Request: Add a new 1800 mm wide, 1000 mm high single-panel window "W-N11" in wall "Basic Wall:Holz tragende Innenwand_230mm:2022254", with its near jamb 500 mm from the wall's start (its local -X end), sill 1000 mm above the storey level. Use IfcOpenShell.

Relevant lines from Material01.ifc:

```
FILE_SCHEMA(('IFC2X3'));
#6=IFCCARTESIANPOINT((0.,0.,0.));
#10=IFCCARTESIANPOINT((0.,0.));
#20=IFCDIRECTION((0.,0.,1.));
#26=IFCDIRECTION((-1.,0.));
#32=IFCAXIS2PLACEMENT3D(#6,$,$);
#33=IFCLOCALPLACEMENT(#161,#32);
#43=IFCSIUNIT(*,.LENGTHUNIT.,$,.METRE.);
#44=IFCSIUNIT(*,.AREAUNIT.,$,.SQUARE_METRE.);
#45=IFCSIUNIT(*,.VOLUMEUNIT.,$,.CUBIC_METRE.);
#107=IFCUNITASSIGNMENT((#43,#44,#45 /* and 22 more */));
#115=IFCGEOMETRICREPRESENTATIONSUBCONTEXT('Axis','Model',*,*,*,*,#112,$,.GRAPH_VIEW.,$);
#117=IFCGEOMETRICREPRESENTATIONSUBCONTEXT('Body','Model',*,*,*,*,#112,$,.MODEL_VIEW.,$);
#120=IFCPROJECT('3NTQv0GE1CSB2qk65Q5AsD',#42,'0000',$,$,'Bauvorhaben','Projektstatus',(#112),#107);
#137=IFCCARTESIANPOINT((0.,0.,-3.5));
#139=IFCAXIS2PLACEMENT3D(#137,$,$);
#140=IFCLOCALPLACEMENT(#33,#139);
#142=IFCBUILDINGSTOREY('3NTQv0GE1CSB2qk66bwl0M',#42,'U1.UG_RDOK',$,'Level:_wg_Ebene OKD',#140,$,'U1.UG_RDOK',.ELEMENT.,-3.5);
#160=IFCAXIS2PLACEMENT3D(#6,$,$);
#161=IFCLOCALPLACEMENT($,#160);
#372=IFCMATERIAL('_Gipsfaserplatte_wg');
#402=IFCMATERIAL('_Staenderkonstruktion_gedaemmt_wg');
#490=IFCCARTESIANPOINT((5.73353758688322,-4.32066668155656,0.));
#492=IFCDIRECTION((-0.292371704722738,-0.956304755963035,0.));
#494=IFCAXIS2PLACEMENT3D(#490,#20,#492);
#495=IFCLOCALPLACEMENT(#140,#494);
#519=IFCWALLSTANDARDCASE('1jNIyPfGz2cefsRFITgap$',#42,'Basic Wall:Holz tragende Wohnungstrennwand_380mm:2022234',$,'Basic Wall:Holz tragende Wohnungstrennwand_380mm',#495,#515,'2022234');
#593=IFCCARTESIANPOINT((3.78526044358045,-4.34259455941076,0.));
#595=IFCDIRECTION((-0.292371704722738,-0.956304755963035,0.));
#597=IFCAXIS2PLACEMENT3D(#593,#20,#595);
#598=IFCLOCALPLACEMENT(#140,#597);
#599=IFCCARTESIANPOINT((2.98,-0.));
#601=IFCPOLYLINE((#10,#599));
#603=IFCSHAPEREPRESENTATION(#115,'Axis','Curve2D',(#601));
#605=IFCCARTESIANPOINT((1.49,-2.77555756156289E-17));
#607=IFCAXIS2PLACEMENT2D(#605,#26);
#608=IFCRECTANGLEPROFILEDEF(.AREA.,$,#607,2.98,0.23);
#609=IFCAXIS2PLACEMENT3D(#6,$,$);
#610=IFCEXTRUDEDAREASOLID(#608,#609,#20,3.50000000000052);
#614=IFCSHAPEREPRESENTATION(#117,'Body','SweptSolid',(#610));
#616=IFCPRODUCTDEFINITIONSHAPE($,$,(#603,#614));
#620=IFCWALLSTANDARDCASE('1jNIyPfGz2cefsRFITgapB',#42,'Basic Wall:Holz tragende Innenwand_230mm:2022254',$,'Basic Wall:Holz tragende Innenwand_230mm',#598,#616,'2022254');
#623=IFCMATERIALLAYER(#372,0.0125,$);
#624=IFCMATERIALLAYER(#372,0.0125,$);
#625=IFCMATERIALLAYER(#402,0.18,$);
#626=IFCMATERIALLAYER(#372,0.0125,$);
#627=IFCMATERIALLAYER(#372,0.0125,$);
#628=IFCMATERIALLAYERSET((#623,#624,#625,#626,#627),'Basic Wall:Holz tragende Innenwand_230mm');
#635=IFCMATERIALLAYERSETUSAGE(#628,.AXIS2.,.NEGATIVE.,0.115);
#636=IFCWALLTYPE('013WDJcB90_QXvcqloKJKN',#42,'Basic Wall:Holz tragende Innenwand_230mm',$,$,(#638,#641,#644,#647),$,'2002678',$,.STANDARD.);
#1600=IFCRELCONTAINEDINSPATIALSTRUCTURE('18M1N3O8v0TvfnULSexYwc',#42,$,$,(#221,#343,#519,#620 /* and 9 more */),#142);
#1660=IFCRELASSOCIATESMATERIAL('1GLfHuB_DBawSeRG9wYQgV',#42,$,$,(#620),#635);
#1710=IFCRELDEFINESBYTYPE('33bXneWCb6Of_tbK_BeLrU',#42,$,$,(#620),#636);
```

```python
import numpy as np
import ifcopenshell
import ifcopenshell.api.feature
import ifcopenshell.api.geometry
import ifcopenshell.api.root
import ifcopenshell.api.spatial
import ifcopenshell.api.type
import ifcopenshell.geom
import ifcopenshell.util.element
import ifcopenshell.util.placement
import ifcopenshell.util.representation
import ifcopenshell.util.shape
import ifcopenshell.util.unit

model = ifcopenshell.open("Material01.ifc")
unit_scale = ifcopenshell.util.unit.calculate_unit_scale(model)
settings = ifcopenshell.geom.settings()


def volume(element):
    """Net volume in cubic metres, openings subtracted."""
    shape = ifcopenshell.geom.create_shape(settings, element)
    return ifcopenshell.util.shape.get_volume(shape.geometry)


wall = model.by_guid("1jNIyPfGz2cefsRFITgapB")
storey = ifcopenshell.util.element.get_container(wall, ifc_class="IfcBuildingStorey")
context = ifcopenshell.util.representation.get_context(model, "Model", "Body", "MODEL_VIEW")
before = volume(wall)

width, height, from_end, sill = 1.8, 1, 0.5, 1  # metres

# The wall runs along its own X axis, and the end named is its -X end.
wall_shape = ifcopenshell.geom.create_shape(settings, wall)
x, y, z = ifcopenshell.util.shape.get_vertices(wall_shape.geometry).T
start = x.min() + from_end
face, thickness = float(y.min()), float(y.max() - y.min())
wall_matrix = ifcopenshell.util.placement.get_local_placement(wall.ObjectPlacement)
level = ifcopenshell.util.placement.get_local_placement(storey.ObjectPlacement)[2, 3]


def in_wall(x, y):
    """Placement at x, y metres in the wall's axes, at sill height."""
    matrix = wall_matrix.copy()
    matrix[:, 3] = wall_matrix @ np.array([x / unit_scale, y / unit_scale, 0.0, 1.0])
    matrix[2, 3] = level + sill / unit_scale
    return matrix


# Opening: a box that overshoots both wall faces by 50 mm.
opening = ifcopenshell.api.root.create_entity(model, ifc_class="IfcOpeningElement")
box = ifcopenshell.api.geometry.add_wall_representation(
    model, context=context, length=width, height=height, thickness=thickness + 0.1
)
ifcopenshell.api.geometry.assign_representation(model, product=opening, representation=box)
ifcopenshell.api.geometry.edit_object_placement(model, product=opening, matrix=in_wall(start, face - 0.05), is_si=False)
ifcopenshell.api.feature.add_feature(model, feature=opening, element=wall)

window = ifcopenshell.api.root.create_entity(model, ifc_class="IfcWindow", name="W-N11")
window.OverallWidth, window.OverallHeight = width / unit_scale, height / unit_scale
body = ifcopenshell.api.geometry.add_window_representation(
    model,
    context=context,
    overall_width=window.OverallWidth,
    overall_height=window.OverallHeight,
    partition_type="SINGLE_PANEL",
)
ifcopenshell.api.geometry.assign_representation(model, product=window, representation=body)
ifcopenshell.api.spatial.assign_container(model, products=[window], relating_structure=storey)
fills = ifcopenshell.api.feature.add_filling(model, opening=opening, element=window)
fills.OwnerHistory = window.OwnerHistory  # required in IFC2X3

# IFC2X3 keeps the operation on the window style.
style = ifcopenshell.api.root.create_entity(model, ifc_class="IfcWindowStyle", name="W-N11")
style.OperationType, style.ConstructionType = "SINGLE_PANEL", "NOTDEFINED"
style.ParameterTakesPrecedence = style.Sizeable = False
ifcopenshell.api.type.assign_type(model, related_objects=[window], relating_type=style)

# Centre the window in the wall's thickness.
ifcopenshell.api.geometry.edit_object_placement(model, product=window, matrix=in_wall(start, face), is_si=False)
window_shape = ifcopenshell.geom.create_shape(settings, window)
depth = ifcopenshell.util.shape.get_vertices(window_shape.geometry)[:, 1]
offset = face + thickness / 2 - (depth.min() + depth.max()) / 2
ifcopenshell.api.geometry.edit_object_placement(model, product=window, matrix=in_wall(start, offset), is_si=False)

after = volume(wall)

print(f"wall volume {before:.3f} -> {after:.3f} m3")

model.write("Material01_v2.ifc")
```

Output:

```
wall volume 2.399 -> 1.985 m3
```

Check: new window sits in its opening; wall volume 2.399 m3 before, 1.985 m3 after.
